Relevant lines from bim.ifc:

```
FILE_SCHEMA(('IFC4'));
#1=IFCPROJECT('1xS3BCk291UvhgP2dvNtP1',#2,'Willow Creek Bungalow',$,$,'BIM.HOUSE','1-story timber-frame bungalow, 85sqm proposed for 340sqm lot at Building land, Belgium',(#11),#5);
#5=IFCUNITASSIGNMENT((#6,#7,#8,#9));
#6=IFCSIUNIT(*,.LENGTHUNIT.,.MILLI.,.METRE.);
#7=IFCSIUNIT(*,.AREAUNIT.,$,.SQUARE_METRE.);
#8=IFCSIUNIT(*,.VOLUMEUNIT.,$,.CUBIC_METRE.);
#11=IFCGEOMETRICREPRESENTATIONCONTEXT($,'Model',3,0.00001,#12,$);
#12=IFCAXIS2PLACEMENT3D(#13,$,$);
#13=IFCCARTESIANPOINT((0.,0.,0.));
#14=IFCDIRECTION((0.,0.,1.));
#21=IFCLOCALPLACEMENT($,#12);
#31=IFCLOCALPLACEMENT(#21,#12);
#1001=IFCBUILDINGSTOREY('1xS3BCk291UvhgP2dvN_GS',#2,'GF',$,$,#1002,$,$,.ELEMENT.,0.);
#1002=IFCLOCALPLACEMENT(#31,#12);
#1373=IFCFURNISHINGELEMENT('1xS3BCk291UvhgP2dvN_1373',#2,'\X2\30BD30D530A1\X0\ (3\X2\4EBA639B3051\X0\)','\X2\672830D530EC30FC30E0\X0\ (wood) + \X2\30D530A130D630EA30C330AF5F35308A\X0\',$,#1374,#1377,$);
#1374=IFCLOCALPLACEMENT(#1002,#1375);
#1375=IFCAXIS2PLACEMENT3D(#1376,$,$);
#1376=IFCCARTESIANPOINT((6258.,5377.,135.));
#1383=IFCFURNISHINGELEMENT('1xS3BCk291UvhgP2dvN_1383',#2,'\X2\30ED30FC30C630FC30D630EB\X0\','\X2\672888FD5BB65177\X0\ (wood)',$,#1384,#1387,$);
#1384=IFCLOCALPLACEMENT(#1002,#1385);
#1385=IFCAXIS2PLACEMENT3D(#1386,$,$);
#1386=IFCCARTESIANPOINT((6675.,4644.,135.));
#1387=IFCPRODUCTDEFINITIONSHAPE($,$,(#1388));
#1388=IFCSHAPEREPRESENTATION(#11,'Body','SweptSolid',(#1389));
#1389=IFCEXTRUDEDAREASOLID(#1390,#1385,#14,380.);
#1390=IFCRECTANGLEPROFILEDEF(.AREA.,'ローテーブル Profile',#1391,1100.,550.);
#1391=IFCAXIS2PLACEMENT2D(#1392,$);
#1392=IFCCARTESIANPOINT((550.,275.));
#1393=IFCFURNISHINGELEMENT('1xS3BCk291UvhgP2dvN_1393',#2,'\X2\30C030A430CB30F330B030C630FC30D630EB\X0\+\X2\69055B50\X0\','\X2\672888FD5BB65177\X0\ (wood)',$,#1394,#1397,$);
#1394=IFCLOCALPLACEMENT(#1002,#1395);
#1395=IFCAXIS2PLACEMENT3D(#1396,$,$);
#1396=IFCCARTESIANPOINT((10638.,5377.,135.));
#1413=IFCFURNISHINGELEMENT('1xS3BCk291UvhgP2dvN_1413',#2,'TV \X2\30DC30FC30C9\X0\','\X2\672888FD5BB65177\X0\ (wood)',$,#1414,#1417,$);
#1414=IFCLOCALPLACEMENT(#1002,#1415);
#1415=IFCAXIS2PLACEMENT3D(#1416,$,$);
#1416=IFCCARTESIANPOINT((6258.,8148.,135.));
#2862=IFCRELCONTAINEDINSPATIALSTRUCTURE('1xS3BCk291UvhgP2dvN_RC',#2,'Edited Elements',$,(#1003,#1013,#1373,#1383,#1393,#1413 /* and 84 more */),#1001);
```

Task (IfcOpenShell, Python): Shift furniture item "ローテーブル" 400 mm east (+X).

```python
import ifcopenshell
import ifcopenshell.api.geometry
import ifcopenshell.util.placement

model = ifcopenshell.open("bim.ifc")

item = model.by_id(1383)
matrix = ifcopenshell.util.placement.get_local_placement(item.ObjectPlacement)
matrix[0, 3] += 400.0
ifcopenshell.api.geometry.edit_object_placement(model, product=item, matrix=matrix, is_si=False)

print(ifcopenshell.util.placement.get_local_placement(item.ObjectPlacement).round(3) + 0.0)

model.write("bim_updated.ifc")
```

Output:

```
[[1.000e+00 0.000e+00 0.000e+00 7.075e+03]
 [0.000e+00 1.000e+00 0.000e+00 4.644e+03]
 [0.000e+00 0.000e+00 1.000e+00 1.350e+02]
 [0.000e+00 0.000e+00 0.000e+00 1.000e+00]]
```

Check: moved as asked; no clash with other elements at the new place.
